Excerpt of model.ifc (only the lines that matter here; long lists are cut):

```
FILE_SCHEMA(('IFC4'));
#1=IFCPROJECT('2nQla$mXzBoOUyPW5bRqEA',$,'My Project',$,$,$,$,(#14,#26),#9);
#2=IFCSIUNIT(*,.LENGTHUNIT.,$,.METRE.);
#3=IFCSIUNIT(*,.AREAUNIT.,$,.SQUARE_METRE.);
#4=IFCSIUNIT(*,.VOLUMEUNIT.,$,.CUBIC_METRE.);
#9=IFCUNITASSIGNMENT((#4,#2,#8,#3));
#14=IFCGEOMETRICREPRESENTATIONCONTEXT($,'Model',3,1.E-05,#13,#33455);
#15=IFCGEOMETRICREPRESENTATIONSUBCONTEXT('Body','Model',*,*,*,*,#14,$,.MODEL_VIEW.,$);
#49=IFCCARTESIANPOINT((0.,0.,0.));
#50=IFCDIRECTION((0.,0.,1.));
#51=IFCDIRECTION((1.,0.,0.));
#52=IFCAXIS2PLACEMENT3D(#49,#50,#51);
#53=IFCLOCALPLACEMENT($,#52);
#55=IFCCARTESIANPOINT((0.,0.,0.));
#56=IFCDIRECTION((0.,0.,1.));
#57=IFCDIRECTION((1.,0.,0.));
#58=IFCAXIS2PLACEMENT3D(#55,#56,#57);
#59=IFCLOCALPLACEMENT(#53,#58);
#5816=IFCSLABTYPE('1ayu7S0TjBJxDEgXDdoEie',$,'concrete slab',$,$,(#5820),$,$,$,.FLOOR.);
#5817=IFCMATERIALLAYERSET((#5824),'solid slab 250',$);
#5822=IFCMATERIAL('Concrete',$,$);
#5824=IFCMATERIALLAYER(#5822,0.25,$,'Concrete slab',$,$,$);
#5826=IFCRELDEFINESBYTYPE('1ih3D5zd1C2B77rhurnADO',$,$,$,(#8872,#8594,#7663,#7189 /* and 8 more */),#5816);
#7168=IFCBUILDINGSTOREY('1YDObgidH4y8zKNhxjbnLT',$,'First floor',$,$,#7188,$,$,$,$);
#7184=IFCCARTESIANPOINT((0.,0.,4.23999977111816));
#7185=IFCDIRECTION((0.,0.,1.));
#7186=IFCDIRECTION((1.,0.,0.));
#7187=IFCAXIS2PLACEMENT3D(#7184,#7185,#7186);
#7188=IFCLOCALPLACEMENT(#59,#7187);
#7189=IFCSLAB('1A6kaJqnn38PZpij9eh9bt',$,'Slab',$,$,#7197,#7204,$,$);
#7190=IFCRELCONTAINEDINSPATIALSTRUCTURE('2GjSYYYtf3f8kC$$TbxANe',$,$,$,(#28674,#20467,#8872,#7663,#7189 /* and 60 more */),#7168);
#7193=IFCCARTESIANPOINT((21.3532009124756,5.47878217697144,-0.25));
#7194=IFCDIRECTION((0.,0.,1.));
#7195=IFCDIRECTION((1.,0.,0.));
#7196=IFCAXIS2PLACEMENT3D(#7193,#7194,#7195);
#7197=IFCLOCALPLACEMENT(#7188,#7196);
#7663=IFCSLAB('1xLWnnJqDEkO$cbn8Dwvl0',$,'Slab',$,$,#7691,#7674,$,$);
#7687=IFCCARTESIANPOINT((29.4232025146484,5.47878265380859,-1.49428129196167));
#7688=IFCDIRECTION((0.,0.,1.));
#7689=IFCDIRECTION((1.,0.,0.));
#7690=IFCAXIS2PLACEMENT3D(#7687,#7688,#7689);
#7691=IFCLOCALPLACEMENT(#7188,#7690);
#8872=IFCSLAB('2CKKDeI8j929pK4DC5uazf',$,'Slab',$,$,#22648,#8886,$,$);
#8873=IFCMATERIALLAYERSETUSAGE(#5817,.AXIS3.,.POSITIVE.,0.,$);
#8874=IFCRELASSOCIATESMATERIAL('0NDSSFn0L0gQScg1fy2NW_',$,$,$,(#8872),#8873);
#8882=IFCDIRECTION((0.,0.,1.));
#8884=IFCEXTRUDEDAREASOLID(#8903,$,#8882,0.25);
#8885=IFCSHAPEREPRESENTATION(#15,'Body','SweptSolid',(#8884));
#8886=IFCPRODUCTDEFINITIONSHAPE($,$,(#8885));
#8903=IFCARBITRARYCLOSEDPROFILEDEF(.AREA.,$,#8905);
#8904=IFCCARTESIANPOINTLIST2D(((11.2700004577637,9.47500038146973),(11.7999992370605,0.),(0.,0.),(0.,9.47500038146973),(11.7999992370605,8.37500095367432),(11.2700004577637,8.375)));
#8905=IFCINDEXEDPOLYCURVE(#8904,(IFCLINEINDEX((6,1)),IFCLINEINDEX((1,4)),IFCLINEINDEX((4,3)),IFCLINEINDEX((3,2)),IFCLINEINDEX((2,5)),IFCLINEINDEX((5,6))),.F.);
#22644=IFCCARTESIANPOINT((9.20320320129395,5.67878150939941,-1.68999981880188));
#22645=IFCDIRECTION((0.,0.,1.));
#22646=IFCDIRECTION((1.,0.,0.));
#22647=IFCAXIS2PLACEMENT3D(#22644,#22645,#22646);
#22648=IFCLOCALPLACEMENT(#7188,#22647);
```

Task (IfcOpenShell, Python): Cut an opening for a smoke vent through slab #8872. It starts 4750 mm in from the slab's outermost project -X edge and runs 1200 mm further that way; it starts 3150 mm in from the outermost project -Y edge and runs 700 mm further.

```python
import numpy as np
import ifcopenshell
import ifcopenshell.api.feature
import ifcopenshell.api.geometry
import ifcopenshell.api.root
import ifcopenshell.geom
import ifcopenshell.util.placement
import ifcopenshell.util.representation
import ifcopenshell.util.shape
import ifcopenshell.util.unit

model = ifcopenshell.open("model.ifc")
unit_scale = ifcopenshell.util.unit.calculate_unit_scale(model)
settings = ifcopenshell.geom.settings()


def volume(element):
    """Net volume in cubic metres, openings subtracted."""
    shape = ifcopenshell.geom.create_shape(settings, element)
    return ifcopenshell.util.shape.get_volume(shape.geometry)


slab = model.by_guid("2CKKDeI8j929pK4DC5uazf")
before = volume(slab)

# Extent in the slab's own axes, in metres. The edges named are its -X and -Y sides.
slab_shape = ifcopenshell.geom.create_shape(settings, slab)
vertices = ifcopenshell.util.shape.get_vertices(slab_shape.geometry)
x_min, y_min, bottom = vertices.min(axis=0)
top = vertices[:, 2].max()

opening = ifcopenshell.api.root.create_entity(model, ifc_class="IfcOpeningElement", name="Smoke vent opening", predefined_type="OPENING")
context = ifcopenshell.util.representation.get_context(model, "Model", "Body", "MODEL_VIEW")
width, depth = 1.2, 0.7
outline = [(0.0, 0.0), (width, 0.0), (width, depth), (0.0, depth), (0.0, 0.0)]
# Overshoot both faces by 50 mm so the cut is clean.
shape = ifcopenshell.api.geometry.add_slab_representation(
    model, context=context, depth=top - bottom + 0.1, polyline=outline
)
ifcopenshell.api.geometry.assign_representation(model, product=opening, representation=shape)

matrix = ifcopenshell.util.placement.get_local_placement(slab.ObjectPlacement)
matrix[:, 3] = matrix @ np.append(np.array([x_min + 4.75, y_min + 3.15, bottom - 0.05]) / unit_scale, 1.0)
ifcopenshell.api.geometry.edit_object_placement(model, product=opening, matrix=matrix, is_si=False)
ifcopenshell.api.feature.add_feature(model, feature=opening, element=slab)

after = volume(slab)

print(f"slab volume {before:.3f} -> {after:.3f} m3")

model.write("model_rev.ifc")
```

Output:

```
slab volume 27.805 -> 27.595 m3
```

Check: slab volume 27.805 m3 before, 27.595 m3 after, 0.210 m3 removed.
